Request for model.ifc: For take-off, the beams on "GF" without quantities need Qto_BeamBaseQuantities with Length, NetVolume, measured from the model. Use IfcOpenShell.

First a look at what the model holds.

```python
import ifcopenshell
import ifcopenshell.util.element
import ifcopenshell.util.unit

model = ifcopenshell.open("model.ifc")
print(model.schema)
for unit_type in ("LENGTHUNIT", "AREAUNIT", "VOLUMEUNIT"):
    print(unit_type, ifcopenshell.util.unit.calculate_unit_scale(model, unit_type))
storey = next(s for s in model.by_type("IfcBuildingStorey") if s.Name == "GF")
beams = [e for e in ifcopenshell.util.element.get_decomposition(storey) if e.is_a("IfcBeam")]
for e in sorted(beams, key=lambda e: e.id()):
    print(e.id(), e.is_a(), e.Name, list(ifcopenshell.util.element.get_psets(e, qtos_only=True)), sep=" | ")
```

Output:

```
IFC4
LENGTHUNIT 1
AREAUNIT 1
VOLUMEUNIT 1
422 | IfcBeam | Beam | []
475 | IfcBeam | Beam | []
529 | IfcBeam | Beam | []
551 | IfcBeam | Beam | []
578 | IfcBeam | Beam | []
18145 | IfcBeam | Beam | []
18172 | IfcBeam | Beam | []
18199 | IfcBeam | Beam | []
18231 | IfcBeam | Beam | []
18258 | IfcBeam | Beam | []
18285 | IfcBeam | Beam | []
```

```python
import ifcopenshell
import ifcopenshell.api.pset
import ifcopenshell.geom
import ifcopenshell.util.element
import ifcopenshell.util.shape
import ifcopenshell.util.unit

model = ifcopenshell.open("model.ifc")
unit_scale = ifcopenshell.util.unit.calculate_unit_scale(model)
volume_scale = ifcopenshell.util.unit.calculate_unit_scale(model, "VOLUMEUNIT")
settings = ifcopenshell.geom.settings()

storey = next(s for s in model.by_type("IfcBuildingStorey") if s.Name == "GF")
beams = [e for e in ifcopenshell.util.element.get_decomposition(storey) if e.is_a("IfcBeam")]

for e in sorted(beams, key=lambda e: e.id()):
    if ifcopenshell.util.element.get_psets(e, qtos_only=True, should_inherit=False):
        continue
    # Geometry comes back in metres, in the element's own axes.
    shape = ifcopenshell.geom.create_shape(settings, e)
    values = {
        "Length": ifcopenshell.util.shape.get_max_xyz(shape.geometry) / unit_scale,
        "NetVolume": ifcopenshell.util.shape.get_volume(shape.geometry) / volume_scale,
    }
    qto = ifcopenshell.api.pset.add_qto(model, product=e, name="Qto_BeamBaseQuantities")
    ifcopenshell.api.pset.edit_qto(model, qto=qto, properties=values)
    print(e.id(), {k: round(v, 3) for k, v in values.items()})

model.write("model_updated.ifc")
```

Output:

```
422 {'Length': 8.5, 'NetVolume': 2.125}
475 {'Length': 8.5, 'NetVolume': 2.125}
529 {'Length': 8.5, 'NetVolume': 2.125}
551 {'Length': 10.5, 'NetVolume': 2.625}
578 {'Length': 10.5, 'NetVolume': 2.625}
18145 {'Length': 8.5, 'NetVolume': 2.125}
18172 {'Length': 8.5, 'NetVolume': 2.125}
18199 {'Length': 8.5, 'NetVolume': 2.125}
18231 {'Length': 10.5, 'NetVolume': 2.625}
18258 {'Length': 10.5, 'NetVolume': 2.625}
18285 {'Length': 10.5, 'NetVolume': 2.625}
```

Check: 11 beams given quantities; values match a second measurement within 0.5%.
